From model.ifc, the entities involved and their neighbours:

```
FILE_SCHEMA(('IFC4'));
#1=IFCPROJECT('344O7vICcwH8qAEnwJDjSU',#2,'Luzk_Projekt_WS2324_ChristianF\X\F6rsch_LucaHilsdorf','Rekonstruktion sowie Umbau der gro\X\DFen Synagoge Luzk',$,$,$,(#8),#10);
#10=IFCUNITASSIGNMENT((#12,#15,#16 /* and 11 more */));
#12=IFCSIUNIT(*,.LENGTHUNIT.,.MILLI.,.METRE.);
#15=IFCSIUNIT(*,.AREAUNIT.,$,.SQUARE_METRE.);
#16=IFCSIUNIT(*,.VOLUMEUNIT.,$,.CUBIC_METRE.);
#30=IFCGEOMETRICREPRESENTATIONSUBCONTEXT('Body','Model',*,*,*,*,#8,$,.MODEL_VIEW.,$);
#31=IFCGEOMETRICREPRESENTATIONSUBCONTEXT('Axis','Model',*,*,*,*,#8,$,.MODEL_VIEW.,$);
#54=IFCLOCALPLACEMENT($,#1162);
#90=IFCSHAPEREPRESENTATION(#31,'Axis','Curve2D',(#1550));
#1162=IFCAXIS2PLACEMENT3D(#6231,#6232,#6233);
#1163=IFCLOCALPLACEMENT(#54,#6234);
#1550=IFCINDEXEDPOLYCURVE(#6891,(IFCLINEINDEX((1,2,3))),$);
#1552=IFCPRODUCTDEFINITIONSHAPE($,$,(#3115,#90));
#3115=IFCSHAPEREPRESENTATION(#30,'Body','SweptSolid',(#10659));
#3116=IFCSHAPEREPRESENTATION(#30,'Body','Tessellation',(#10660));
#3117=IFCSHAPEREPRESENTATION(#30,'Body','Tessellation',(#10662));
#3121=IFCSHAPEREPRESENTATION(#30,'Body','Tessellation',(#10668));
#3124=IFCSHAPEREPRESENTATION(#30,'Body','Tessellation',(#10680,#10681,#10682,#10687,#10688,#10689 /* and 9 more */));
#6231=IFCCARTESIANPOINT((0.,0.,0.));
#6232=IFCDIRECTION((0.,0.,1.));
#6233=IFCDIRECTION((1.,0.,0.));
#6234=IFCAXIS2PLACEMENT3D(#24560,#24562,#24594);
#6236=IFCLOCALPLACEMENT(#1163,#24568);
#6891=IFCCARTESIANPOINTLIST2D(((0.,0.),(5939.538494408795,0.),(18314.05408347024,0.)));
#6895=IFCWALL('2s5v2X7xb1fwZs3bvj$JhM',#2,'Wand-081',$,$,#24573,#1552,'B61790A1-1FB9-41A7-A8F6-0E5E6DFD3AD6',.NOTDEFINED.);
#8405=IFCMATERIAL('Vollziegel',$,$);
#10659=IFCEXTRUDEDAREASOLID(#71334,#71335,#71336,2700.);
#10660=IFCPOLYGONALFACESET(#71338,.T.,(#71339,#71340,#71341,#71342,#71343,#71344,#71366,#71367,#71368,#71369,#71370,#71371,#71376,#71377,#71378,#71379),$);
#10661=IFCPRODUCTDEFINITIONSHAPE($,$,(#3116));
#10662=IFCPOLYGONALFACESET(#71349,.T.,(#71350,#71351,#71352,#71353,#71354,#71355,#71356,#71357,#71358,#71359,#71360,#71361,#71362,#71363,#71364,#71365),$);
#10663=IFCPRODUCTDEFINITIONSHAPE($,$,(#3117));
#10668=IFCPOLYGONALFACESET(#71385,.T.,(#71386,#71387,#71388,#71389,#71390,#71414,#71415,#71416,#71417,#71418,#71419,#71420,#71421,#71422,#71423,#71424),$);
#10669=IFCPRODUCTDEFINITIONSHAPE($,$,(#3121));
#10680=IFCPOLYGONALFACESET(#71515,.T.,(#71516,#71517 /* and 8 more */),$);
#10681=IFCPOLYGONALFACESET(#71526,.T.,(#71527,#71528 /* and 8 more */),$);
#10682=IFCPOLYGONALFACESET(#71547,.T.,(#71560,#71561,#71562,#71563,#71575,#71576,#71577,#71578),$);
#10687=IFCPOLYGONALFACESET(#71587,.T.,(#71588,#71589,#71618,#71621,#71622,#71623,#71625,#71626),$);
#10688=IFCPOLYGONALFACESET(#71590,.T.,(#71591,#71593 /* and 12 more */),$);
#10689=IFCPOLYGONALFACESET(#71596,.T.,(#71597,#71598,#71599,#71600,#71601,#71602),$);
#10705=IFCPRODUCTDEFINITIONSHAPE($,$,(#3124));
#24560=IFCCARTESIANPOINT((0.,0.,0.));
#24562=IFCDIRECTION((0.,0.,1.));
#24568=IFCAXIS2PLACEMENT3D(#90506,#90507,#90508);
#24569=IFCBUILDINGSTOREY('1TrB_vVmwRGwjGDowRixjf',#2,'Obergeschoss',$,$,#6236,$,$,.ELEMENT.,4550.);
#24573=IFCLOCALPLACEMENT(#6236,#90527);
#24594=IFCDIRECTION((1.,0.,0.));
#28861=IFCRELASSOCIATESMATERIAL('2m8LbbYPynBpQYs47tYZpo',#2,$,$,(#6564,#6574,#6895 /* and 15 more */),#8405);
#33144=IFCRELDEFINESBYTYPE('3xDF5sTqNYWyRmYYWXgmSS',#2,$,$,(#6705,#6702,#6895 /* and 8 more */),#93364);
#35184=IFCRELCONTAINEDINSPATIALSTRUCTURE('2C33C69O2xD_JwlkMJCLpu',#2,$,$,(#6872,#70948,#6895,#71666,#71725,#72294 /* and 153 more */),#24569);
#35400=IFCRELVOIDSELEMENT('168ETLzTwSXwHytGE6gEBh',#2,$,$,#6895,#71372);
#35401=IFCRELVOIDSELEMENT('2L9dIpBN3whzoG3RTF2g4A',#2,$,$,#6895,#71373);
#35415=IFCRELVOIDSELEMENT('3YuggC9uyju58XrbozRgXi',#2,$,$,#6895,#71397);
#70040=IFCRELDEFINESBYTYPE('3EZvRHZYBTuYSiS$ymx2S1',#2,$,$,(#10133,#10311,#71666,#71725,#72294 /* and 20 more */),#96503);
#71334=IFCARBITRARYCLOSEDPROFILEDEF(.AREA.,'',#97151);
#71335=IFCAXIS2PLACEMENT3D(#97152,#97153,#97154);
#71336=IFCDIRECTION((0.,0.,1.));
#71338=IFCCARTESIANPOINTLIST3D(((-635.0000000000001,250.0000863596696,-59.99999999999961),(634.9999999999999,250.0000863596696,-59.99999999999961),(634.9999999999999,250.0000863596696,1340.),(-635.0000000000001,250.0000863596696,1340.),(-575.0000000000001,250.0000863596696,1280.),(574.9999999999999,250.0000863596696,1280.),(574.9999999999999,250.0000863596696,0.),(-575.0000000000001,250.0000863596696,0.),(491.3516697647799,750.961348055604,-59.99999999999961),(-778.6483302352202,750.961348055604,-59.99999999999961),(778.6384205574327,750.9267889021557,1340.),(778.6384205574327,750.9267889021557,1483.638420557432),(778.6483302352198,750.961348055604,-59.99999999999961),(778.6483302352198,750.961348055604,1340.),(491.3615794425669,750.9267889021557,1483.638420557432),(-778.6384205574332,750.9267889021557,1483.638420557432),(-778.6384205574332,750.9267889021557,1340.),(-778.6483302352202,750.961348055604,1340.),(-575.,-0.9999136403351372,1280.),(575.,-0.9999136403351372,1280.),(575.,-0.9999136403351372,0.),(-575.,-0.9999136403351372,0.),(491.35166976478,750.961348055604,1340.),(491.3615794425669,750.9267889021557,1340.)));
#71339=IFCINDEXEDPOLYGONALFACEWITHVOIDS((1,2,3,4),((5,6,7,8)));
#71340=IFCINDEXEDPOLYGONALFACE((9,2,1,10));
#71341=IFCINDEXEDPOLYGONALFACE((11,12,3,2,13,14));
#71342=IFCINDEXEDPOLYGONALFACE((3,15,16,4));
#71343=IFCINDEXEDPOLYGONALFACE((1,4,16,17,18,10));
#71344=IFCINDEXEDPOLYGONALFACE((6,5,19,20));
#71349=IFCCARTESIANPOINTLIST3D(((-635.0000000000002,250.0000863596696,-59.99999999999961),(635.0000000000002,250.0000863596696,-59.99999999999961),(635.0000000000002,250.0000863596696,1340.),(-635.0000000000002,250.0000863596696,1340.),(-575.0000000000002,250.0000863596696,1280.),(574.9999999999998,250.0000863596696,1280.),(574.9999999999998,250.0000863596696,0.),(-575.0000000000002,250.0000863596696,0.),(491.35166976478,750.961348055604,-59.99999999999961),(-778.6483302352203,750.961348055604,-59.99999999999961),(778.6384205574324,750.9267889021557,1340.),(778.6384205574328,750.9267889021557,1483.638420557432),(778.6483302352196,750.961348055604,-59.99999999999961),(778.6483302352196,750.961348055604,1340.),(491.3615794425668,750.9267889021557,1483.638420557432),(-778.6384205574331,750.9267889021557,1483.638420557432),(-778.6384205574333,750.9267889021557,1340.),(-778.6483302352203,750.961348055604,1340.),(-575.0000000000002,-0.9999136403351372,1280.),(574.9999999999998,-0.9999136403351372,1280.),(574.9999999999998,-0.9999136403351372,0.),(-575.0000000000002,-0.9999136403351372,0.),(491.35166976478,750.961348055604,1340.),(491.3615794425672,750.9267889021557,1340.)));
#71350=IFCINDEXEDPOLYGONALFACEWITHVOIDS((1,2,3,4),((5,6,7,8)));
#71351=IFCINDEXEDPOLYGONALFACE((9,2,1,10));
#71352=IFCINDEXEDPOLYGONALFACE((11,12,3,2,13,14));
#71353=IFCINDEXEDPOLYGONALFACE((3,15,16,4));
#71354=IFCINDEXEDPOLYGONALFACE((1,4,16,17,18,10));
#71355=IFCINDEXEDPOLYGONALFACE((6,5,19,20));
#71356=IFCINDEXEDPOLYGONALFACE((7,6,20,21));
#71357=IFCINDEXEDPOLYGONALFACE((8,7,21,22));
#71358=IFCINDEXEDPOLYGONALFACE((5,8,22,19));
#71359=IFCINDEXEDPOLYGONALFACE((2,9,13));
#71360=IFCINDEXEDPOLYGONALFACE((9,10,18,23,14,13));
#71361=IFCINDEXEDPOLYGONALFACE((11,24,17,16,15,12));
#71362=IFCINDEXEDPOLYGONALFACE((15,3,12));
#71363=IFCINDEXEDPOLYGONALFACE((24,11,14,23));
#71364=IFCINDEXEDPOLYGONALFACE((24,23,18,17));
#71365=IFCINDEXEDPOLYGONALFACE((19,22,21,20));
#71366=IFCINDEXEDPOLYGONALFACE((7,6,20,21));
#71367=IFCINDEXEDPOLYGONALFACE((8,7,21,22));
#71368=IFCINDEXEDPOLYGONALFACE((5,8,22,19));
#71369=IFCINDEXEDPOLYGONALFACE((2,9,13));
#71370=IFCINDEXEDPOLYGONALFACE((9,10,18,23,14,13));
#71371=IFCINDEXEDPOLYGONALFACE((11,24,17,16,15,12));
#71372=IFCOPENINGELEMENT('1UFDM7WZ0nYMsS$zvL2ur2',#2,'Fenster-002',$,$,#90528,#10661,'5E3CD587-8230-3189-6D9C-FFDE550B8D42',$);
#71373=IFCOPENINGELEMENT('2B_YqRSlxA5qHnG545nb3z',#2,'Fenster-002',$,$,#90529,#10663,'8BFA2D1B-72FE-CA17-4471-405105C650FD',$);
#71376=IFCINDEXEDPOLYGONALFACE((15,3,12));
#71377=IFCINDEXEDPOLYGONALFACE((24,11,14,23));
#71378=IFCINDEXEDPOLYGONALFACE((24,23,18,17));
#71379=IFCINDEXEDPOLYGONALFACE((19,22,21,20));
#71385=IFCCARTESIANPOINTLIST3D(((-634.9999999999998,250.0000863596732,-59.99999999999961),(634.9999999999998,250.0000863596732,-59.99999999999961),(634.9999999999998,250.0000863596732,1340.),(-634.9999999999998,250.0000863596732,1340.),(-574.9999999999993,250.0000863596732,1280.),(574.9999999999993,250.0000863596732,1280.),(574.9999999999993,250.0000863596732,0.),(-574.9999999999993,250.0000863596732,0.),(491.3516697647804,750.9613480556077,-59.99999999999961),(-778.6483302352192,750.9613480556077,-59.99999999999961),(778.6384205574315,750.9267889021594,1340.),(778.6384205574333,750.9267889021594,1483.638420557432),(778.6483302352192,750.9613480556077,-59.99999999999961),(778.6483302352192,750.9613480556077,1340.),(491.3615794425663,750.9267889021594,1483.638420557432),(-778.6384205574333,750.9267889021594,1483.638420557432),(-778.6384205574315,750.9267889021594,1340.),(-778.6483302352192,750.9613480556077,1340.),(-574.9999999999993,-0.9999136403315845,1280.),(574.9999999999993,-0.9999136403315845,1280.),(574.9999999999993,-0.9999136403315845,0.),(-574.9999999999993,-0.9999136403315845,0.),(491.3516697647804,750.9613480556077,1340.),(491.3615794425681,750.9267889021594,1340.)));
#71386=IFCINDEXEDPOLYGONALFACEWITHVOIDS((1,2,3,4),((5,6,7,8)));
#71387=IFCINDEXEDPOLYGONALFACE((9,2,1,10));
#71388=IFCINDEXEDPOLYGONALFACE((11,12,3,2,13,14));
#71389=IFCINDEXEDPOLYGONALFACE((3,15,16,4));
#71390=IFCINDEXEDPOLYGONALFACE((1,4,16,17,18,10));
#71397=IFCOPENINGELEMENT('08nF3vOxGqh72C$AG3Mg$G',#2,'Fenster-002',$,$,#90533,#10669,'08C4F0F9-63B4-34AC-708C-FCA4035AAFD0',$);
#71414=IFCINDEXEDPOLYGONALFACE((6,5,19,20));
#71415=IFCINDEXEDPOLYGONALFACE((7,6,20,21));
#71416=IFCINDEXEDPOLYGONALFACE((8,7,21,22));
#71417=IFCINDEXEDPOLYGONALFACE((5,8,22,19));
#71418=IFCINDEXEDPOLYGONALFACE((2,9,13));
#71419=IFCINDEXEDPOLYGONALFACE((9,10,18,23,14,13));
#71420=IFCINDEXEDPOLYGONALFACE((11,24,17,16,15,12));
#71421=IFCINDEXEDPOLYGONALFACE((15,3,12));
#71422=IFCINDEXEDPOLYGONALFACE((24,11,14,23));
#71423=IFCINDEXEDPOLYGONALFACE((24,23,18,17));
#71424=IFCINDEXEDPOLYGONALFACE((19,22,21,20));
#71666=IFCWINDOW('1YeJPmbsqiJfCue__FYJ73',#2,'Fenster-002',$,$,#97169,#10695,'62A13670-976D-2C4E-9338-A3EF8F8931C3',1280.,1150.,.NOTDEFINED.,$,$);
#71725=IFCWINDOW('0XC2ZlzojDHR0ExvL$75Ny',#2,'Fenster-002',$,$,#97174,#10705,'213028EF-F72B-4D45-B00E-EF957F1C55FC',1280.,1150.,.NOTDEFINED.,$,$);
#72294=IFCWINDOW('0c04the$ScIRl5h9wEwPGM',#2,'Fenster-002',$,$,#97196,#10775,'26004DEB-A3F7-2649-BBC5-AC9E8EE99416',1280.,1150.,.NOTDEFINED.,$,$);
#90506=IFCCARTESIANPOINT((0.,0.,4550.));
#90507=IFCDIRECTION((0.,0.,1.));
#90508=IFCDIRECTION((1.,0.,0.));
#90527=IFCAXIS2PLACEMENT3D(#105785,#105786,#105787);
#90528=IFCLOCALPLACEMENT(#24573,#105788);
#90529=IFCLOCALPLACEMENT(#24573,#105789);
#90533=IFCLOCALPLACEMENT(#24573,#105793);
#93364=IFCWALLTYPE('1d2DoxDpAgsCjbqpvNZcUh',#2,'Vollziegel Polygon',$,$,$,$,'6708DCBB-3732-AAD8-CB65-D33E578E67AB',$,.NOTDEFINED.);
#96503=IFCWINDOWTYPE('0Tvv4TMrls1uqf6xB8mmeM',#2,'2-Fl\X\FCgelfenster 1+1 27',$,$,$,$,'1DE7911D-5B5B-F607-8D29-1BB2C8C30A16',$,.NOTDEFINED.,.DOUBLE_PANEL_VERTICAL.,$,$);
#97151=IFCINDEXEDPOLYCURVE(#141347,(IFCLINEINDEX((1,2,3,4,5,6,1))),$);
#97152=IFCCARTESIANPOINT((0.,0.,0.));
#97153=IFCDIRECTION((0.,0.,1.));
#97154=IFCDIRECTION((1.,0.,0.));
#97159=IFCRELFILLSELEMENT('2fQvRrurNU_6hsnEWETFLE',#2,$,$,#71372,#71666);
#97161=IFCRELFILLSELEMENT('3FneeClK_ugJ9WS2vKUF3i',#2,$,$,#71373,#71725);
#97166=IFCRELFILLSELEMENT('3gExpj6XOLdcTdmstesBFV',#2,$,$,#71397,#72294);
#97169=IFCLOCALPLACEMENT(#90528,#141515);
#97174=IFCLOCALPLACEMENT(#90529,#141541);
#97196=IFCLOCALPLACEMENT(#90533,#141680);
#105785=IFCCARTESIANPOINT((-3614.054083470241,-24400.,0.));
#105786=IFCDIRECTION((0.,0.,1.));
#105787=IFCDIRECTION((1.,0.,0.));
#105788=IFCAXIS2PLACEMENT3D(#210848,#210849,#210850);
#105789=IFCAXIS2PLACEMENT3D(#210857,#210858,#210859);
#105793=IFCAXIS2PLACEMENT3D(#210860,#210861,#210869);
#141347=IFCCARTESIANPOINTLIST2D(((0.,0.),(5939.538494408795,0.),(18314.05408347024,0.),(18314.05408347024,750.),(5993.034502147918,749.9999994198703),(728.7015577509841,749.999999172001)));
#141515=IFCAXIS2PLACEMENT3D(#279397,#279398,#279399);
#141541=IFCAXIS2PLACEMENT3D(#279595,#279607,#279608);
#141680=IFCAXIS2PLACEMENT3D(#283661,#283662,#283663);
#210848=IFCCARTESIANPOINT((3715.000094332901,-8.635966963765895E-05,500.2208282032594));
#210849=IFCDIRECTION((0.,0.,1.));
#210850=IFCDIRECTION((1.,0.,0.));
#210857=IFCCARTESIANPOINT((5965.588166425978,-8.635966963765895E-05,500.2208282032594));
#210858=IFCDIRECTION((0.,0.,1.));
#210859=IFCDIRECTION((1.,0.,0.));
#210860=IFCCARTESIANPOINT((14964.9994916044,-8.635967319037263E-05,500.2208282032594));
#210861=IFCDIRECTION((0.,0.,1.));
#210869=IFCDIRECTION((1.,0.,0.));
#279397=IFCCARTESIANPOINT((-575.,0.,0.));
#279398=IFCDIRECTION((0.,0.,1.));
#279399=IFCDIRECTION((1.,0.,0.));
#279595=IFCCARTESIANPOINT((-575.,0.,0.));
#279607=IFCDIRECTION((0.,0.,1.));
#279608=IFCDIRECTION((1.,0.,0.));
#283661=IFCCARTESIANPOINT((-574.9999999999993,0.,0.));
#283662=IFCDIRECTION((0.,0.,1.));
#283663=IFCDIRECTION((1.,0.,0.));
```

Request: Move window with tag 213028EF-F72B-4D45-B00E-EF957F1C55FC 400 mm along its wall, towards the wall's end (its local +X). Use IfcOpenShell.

```python
import ifcopenshell
import ifcopenshell.api.geometry
import ifcopenshell.util.placement
import ifcopenshell.util.unit

model = ifcopenshell.open("model.ifc")
unit_scale = ifcopenshell.util.unit.calculate_unit_scale(model)

window = model.by_guid("0XC2ZlzojDHR0ExvL$75Ny")
opening = window.FillsVoids[0].RelatingOpeningElement
wall = opening.VoidsElements[0].RelatingBuildingElement

wall_matrix = ifcopenshell.util.placement.get_local_placement(wall.ObjectPlacement)
shift = wall_matrix[:3, 0] * 0.4 / unit_scale
before = ifcopenshell.util.placement.get_local_placement(window.ObjectPlacement)[:3, 3].copy()

# The window is placed relative to its opening, so it follows when the opening moves.
matrix = ifcopenshell.util.placement.get_local_placement(opening.ObjectPlacement)
matrix[:3, 3] += shift
ifcopenshell.api.geometry.edit_object_placement(
    model, product=opening, matrix=matrix, is_si=False, should_transform_children=True
)

after = ifcopenshell.util.placement.get_local_placement(window.ObjectPlacement)[:3, 3]
print("window moved by", (after - before).round(3) + 0.0)

model.write("model_v2.ifc")
```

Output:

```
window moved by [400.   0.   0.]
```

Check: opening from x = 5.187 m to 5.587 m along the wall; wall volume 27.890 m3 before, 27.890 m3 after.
